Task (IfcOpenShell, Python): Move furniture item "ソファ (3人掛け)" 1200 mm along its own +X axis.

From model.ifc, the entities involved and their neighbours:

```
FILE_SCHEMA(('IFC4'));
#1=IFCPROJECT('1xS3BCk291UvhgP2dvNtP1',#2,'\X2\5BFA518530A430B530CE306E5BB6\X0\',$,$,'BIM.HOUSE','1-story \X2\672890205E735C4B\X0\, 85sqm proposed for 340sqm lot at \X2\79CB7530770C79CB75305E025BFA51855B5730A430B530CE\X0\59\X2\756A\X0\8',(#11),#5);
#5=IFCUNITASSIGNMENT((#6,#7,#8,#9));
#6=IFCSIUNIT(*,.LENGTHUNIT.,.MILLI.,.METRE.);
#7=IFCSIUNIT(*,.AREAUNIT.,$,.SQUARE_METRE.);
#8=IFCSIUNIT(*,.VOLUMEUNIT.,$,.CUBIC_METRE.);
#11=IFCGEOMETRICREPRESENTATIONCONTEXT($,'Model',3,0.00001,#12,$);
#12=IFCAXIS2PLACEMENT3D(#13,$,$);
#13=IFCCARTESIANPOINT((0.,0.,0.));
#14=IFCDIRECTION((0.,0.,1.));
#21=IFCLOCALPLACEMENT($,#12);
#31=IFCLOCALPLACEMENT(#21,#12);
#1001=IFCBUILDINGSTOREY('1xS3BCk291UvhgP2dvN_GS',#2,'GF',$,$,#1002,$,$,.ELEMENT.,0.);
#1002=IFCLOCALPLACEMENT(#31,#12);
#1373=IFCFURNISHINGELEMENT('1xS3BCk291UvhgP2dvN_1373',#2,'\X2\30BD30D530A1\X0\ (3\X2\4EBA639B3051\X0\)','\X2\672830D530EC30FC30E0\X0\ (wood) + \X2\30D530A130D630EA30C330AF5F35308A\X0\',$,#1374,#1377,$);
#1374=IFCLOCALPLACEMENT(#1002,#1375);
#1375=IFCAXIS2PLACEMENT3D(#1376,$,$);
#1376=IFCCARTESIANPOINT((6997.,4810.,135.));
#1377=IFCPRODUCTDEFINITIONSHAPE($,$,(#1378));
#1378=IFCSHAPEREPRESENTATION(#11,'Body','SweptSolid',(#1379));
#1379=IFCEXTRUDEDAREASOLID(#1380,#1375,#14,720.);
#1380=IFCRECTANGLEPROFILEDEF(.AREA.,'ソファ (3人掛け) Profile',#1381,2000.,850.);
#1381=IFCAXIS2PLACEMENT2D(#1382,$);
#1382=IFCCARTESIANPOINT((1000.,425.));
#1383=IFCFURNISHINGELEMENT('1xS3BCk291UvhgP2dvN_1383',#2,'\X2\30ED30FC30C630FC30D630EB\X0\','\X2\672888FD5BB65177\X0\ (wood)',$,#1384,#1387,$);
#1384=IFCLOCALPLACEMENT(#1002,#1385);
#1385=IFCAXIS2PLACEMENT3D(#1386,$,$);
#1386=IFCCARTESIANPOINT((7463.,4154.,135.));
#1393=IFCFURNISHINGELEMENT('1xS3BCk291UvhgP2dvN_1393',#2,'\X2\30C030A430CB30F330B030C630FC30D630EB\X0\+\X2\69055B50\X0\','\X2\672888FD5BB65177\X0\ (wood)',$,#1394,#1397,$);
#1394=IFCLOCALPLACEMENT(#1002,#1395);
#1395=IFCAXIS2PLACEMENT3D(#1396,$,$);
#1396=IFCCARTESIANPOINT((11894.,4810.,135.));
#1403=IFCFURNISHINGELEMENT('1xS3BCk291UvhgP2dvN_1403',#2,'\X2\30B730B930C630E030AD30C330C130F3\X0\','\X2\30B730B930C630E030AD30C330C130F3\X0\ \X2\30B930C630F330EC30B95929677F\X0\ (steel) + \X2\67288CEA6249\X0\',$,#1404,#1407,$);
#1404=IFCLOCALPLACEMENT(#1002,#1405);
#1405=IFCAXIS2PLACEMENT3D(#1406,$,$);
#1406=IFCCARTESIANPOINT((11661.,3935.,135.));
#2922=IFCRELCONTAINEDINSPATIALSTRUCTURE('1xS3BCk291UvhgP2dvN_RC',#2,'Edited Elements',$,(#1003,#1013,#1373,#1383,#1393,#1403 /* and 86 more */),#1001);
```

```python
import ifcopenshell
import ifcopenshell.api.geometry
import ifcopenshell.util.placement

model = ifcopenshell.open("model.ifc")

item = model.by_guid("1xS3BCk291UvhgP2dvN_1373")
matrix = ifcopenshell.util.placement.get_local_placement(item.ObjectPlacement)
matrix[:3, 3] += matrix[:3, 0] * 1200.0
ifcopenshell.api.geometry.edit_object_placement(model, product=item, matrix=matrix, is_si=False)

print(ifcopenshell.util.placement.get_local_placement(item.ObjectPlacement).round(3) + 0.0)

model.write("model_edited.ifc")
```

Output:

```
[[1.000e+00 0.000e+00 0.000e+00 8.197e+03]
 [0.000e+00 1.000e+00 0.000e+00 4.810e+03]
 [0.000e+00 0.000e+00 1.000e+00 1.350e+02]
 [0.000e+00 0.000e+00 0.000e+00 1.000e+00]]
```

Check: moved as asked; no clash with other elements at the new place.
